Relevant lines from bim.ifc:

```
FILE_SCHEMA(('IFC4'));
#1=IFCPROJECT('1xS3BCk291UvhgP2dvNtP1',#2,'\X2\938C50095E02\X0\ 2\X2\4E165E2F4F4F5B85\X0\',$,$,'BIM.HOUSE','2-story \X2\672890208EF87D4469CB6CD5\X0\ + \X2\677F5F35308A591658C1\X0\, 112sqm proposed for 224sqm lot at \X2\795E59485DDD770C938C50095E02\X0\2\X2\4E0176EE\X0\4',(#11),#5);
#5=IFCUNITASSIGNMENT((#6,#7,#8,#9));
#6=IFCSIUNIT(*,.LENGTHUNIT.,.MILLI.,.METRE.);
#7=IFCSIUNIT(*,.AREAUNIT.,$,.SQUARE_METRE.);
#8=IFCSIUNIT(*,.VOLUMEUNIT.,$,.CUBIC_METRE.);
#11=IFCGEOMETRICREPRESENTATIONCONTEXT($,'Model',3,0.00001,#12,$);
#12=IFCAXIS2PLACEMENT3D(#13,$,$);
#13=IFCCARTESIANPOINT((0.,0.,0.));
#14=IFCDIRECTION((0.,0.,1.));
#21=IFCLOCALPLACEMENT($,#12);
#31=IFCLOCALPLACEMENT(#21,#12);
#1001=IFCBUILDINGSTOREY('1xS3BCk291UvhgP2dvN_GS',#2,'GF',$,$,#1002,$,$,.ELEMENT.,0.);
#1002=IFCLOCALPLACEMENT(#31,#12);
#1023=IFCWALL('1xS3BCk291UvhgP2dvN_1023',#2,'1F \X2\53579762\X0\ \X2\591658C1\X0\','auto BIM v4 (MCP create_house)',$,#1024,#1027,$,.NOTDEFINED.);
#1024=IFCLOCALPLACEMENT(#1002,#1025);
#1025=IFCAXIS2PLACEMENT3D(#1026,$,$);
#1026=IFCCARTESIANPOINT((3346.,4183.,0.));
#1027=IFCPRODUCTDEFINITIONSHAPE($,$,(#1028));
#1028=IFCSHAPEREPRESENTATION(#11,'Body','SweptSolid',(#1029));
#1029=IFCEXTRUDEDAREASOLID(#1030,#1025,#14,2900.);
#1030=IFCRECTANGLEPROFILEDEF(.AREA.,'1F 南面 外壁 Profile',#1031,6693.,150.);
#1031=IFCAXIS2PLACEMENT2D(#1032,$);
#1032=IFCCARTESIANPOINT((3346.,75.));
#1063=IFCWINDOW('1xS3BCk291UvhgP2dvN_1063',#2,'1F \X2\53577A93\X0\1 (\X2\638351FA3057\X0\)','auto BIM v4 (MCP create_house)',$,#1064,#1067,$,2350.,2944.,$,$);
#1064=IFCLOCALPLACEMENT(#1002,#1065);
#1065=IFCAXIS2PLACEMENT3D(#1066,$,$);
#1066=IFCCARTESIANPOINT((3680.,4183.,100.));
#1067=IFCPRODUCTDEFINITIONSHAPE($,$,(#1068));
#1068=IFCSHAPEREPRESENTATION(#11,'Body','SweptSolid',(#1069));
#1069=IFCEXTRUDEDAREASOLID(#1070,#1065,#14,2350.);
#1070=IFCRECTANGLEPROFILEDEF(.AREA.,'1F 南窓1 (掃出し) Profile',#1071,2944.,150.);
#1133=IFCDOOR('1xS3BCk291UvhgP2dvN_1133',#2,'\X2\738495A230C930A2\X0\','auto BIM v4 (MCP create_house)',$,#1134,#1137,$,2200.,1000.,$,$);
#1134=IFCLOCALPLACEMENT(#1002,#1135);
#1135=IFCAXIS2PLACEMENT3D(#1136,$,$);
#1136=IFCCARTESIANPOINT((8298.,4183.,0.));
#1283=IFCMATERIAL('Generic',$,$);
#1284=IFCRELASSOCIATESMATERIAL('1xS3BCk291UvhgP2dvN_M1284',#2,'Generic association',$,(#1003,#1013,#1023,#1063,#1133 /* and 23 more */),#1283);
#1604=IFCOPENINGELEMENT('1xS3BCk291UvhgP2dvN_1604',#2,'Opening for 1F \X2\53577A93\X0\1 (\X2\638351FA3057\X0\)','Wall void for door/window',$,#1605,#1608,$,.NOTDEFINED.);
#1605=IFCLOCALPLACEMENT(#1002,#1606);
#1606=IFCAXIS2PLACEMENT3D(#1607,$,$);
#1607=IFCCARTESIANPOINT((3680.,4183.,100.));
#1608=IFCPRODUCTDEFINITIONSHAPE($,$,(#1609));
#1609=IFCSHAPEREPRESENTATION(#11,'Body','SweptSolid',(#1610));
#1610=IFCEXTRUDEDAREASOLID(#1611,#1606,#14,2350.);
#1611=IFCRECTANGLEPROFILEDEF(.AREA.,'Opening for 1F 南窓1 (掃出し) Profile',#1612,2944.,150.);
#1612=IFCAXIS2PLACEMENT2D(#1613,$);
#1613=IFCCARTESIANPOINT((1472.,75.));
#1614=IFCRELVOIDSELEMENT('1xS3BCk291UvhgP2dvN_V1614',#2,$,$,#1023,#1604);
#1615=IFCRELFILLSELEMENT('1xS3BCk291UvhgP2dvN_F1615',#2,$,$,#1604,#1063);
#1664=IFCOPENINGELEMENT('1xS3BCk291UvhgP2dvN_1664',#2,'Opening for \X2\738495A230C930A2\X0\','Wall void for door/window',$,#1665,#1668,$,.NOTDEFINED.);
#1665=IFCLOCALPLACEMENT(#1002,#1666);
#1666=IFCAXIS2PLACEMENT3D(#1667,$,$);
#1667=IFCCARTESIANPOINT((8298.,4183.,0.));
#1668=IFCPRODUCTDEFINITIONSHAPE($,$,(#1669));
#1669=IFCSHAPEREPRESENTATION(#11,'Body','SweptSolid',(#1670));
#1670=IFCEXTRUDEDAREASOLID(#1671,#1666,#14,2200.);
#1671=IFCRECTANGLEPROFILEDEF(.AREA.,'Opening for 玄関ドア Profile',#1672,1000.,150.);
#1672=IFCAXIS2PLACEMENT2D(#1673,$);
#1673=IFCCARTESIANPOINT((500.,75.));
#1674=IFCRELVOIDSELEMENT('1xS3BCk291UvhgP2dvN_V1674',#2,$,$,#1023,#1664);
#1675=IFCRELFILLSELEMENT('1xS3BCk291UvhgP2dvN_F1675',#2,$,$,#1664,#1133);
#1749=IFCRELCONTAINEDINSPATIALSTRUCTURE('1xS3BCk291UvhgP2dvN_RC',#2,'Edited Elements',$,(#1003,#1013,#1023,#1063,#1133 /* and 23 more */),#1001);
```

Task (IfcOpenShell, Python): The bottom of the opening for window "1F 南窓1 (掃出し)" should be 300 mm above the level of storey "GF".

```python
import numpy as np
import ifcopenshell
import ifcopenshell.api.geometry
import ifcopenshell.geom
import ifcopenshell.util.element
import ifcopenshell.util.placement
import ifcopenshell.util.shape
import ifcopenshell.util.unit

model = ifcopenshell.open("bim.ifc")
unit_scale = ifcopenshell.util.unit.calculate_unit_scale(model)

window = model.by_guid("1xS3BCk291UvhgP2dvN_1063")
opening = window.FillsVoids[0].RelatingOpeningElement
storey = ifcopenshell.util.element.get_container(window, ifc_class="IfcBuildingStorey")
level = ifcopenshell.util.placement.get_local_placement(storey.ObjectPlacement)[2, 3]

# The opening's origin need not be at the sill, so measure its lowest point.
shape = ifcopenshell.geom.create_shape(ifcopenshell.geom.settings(), opening)
bottom = ifcopenshell.util.shape.get_shape_bottom_elevation(shape, shape.geometry) / unit_scale
dz = level + 0.3 / unit_scale - bottom

shift = np.array([0.0, 0.0, dz])
# The window is not placed relative to its opening, so move both.
for product in (opening, window):
    matrix = ifcopenshell.util.placement.get_local_placement(product.ObjectPlacement)
    matrix[:3, 3] += shift
    ifcopenshell.api.geometry.edit_object_placement(model, product=product, matrix=matrix, is_si=False)

print(f"moved by {dz * unit_scale:+.3f} m")

model.write("bim_edited.ifc")
```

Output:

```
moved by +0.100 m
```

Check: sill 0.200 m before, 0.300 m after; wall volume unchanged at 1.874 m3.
